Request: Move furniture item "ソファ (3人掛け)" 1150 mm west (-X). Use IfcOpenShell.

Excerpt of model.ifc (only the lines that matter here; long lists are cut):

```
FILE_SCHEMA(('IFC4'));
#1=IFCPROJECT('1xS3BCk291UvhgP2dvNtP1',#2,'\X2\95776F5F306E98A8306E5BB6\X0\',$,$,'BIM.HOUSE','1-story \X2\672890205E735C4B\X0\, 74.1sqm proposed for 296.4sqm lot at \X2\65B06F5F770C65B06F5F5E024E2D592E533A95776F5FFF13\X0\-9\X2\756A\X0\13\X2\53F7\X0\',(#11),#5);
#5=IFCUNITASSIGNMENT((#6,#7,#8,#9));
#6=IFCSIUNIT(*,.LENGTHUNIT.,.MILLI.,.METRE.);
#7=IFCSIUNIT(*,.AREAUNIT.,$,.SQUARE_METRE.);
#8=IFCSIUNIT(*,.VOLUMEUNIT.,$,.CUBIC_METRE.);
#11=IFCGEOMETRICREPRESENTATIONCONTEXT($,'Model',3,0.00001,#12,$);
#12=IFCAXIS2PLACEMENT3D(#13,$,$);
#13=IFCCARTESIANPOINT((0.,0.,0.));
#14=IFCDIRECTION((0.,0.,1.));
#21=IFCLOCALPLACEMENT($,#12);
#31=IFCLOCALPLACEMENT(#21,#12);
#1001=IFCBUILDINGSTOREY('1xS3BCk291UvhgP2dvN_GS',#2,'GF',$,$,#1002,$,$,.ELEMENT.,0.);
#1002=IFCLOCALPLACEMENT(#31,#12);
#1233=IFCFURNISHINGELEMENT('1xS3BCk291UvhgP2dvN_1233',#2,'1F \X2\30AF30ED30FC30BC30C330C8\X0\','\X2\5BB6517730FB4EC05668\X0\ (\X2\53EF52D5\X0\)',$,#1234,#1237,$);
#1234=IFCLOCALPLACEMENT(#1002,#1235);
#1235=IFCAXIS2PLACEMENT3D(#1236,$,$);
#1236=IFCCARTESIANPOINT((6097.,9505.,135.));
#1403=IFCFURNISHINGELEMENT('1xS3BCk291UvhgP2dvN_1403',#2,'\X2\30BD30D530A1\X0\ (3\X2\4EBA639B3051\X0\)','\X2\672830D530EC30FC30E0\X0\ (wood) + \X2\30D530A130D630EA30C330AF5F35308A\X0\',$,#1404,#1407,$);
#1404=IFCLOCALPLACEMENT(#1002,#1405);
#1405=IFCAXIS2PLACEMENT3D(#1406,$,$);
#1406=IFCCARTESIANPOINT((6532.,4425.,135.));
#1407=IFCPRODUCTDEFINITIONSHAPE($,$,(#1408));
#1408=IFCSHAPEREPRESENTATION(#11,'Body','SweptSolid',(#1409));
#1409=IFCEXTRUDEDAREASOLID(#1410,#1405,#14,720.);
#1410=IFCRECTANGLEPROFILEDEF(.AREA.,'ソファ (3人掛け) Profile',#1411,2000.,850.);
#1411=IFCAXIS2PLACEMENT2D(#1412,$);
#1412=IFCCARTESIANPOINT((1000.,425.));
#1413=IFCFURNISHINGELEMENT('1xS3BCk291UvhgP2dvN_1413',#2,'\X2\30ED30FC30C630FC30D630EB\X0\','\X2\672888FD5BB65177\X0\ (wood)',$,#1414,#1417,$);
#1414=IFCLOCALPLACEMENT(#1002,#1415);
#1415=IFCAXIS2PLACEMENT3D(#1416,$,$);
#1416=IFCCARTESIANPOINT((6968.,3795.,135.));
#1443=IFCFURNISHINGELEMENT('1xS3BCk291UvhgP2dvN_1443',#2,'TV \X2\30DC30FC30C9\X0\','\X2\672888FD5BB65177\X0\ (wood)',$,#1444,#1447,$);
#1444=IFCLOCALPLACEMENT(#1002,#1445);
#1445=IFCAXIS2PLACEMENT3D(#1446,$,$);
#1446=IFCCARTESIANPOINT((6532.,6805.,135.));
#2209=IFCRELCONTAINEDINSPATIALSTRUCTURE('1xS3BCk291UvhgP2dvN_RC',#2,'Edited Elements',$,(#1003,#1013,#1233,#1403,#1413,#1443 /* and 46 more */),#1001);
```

```python
import ifcopenshell
import ifcopenshell.api.geometry
import ifcopenshell.util.placement
import ifcopenshell.util.unit

model = ifcopenshell.open("model.ifc")
unit_scale = ifcopenshell.util.unit.calculate_unit_scale(model)

item = model.by_guid("1xS3BCk291UvhgP2dvN_1403")
matrix = ifcopenshell.util.placement.get_local_placement(item.ObjectPlacement)
matrix[0, 3] -= 1.15 / unit_scale
ifcopenshell.api.geometry.edit_object_placement(model, product=item, matrix=matrix, is_si=False)

print(ifcopenshell.util.placement.get_local_placement(item.ObjectPlacement).round(3) + 0.0)

model.write("model_updated.ifc")
```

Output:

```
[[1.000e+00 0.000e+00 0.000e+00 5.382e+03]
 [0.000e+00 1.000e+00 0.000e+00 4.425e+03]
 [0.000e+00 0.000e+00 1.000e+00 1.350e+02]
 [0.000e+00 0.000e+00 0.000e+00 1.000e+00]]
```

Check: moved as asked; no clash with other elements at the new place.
